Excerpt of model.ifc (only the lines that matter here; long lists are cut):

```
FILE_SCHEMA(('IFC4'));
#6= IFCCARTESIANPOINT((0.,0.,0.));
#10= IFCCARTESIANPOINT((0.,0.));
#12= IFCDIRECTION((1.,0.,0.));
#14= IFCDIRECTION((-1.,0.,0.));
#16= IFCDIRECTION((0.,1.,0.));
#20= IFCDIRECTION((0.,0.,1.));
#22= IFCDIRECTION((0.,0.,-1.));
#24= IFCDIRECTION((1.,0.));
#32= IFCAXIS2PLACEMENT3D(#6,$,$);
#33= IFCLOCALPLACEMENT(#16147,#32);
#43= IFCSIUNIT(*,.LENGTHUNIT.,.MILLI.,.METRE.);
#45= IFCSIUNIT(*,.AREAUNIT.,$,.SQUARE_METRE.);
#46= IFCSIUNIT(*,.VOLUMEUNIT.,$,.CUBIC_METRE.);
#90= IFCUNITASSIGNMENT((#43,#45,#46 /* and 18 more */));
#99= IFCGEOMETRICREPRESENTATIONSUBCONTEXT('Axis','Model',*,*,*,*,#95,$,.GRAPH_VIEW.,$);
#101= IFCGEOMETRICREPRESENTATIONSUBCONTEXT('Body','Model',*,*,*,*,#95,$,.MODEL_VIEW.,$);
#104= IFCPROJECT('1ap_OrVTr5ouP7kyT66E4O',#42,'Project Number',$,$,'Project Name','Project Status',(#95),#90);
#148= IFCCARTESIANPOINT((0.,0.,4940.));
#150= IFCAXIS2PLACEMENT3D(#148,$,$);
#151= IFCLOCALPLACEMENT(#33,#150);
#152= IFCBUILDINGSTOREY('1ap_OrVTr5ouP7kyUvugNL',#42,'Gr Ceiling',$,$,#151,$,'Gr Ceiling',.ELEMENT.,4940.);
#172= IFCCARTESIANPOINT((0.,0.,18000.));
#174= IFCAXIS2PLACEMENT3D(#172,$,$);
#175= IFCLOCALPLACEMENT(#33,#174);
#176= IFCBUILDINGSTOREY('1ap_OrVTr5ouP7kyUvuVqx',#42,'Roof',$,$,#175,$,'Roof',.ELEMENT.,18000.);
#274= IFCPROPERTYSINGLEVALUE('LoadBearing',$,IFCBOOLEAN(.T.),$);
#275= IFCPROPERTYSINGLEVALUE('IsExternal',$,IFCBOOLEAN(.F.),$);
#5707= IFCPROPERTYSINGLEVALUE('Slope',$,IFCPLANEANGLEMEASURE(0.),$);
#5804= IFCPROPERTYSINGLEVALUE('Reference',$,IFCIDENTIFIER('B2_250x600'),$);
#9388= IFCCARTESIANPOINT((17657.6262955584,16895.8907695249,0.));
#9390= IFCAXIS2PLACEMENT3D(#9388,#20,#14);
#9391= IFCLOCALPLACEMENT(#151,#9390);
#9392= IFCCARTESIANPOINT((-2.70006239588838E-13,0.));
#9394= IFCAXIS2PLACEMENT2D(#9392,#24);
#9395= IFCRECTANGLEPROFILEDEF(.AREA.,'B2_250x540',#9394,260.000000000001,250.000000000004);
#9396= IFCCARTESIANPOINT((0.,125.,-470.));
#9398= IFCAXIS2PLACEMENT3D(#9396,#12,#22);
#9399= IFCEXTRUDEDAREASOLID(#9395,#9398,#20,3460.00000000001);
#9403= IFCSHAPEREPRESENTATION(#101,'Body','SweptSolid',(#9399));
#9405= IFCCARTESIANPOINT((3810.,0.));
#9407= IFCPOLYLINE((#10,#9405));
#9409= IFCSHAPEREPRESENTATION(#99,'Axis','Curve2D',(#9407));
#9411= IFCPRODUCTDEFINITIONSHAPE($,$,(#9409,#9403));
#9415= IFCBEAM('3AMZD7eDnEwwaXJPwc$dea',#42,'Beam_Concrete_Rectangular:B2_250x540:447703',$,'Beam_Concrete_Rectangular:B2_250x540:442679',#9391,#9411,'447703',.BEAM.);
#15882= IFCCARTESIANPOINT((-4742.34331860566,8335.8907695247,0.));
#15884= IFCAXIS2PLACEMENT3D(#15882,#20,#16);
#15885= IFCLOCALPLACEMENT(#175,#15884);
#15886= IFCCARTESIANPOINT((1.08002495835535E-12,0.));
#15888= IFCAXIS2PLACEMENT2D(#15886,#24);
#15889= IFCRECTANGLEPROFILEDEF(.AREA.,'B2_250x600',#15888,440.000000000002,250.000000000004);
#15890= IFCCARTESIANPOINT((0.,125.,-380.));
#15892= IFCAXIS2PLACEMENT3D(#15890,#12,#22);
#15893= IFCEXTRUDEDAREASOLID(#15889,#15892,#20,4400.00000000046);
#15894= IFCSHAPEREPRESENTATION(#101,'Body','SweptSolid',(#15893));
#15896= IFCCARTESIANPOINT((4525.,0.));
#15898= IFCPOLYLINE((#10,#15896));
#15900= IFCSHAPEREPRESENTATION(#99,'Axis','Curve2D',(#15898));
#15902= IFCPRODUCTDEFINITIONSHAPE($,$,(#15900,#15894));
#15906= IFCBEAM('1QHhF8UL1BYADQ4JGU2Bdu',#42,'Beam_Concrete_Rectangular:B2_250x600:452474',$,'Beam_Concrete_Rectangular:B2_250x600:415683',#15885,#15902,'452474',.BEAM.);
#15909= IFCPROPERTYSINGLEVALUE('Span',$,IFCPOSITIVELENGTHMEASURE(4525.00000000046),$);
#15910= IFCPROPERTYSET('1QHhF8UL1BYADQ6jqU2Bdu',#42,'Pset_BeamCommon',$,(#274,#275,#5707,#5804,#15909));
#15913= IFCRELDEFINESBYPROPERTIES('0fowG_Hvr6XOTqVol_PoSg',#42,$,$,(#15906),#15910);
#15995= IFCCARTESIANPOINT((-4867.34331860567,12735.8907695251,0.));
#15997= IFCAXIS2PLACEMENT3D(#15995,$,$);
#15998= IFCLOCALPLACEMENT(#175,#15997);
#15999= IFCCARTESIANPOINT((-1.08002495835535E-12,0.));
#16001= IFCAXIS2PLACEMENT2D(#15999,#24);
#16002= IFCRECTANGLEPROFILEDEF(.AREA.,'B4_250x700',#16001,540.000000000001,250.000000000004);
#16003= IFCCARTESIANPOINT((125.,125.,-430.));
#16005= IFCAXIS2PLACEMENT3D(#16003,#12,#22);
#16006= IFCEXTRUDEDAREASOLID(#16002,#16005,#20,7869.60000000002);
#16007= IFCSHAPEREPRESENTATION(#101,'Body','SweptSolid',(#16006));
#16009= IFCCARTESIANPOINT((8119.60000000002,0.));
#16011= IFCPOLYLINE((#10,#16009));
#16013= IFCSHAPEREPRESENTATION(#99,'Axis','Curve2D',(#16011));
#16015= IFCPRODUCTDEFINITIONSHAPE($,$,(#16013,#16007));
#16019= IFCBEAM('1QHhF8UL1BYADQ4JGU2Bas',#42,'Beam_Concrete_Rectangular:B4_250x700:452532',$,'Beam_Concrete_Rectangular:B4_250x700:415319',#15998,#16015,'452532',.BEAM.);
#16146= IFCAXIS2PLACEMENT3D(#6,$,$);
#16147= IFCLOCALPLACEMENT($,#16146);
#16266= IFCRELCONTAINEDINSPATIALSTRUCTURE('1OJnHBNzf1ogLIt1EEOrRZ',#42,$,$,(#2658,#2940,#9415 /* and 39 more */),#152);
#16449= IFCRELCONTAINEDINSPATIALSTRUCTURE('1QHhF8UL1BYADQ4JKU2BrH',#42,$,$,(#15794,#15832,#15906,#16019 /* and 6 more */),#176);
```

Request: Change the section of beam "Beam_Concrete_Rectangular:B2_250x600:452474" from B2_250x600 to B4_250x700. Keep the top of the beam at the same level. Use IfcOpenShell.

```python
import ifcopenshell
import ifcopenshell.api.pset
import ifcopenshell.util.element
import ifcopenshell.util.representation

model = ifcopenshell.open("model.ifc")

member = model.by_guid("1QHhF8UL1BYADQ4JGU2Bdu")
source = next(p for p in model.by_type("IfcRectangleProfileDef") if p.ProfileName == "B4_250x700")

body = ifcopenshell.util.representation.get_representation(member, "Model", "Body")
solid = body.Items[0]
old_profile = solid.SweptArea

# Copy the section's sizes but keep this member's own profile position.
profile = ifcopenshell.util.element.copy(model, source)
# Profiles are centred, so shift by half the change in depth to hold the top.
shift = (old_profile.XDim - profile.XDim) / 2
x, y = old_profile.Position.Location.Coordinates
up = (-1.0, 0.0)  # upwards, in the solid's own plane
location = model.createIfcCartesianPoint((x + up[0] * shift, y + up[1] * shift))
profile.Position = model.createIfcAxis2Placement2D(location, old_profile.Position.RefDirection)
solid.SweptArea = profile
if not model.get_total_inverses(old_profile):
    ifcopenshell.util.element.remove_deep2(model, old_profile)
member.Name = member.Name.replace("B2_250x600", "B4_250x700")
member.ObjectType = member.ObjectType.replace("B2_250x600", "B4_250x700")
pset = model.by_id(ifcopenshell.util.element.get_pset(member, "Pset_BeamCommon", should_inherit=False)["id"])
ifcopenshell.api.pset.edit_pset(model, pset=pset, properties={"Reference": "B4_250x700"})

print(solid.SweptArea)

model.write("model_updated.ifc")
```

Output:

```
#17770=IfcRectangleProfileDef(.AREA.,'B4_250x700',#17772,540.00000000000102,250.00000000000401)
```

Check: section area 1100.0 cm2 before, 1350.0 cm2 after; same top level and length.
